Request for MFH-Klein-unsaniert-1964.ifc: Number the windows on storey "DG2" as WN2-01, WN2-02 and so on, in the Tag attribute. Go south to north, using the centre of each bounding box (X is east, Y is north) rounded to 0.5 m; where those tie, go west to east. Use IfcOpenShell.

First a look at what the model holds.

```python
import ifcopenshell
import ifcopenshell.util.element
import ifcopenshell.util.placement

model = ifcopenshell.open("MFH-Klein-unsaniert-1964.ifc")
print(model.schema)
storey = next(s for s in model.by_type("IfcBuildingStorey") if s.Name == "DG2")
windows = [e for e in ifcopenshell.util.element.get_decomposition(storey) if e.is_a("IfcWindow")]
for e in sorted(windows, key=lambda e: e.id()):
    origin = ifcopenshell.util.placement.get_local_placement(e.ObjectPlacement)[:3, 3]
    print(e.id(), e.Tag, e.Name, origin.round(2) + 0.0, sep=" | ")
```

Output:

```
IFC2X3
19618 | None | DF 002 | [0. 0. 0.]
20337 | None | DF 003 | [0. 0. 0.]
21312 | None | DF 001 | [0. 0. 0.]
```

```python
import ifcopenshell
import ifcopenshell.geom
import ifcopenshell.util.element
import ifcopenshell.util.shape

model = ifcopenshell.open("MFH-Klein-unsaniert-1964.ifc")
settings = ifcopenshell.geom.settings()
settings.set("use-world-coords", True)


def centre(element):
    shape = ifcopenshell.geom.create_shape(settings, element)
    return ifcopenshell.util.shape.get_bbox_centroid(shape.geometry)


storey = next(s for s in model.by_type("IfcBuildingStorey") if s.Name == "DG2")
windows = [e for e in ifcopenshell.util.element.get_decomposition(storey) if e.is_a("IfcWindow")]

# Insertion points can sit at a corner or the storey origin, so sort by the geometry (in metres).
centres = {e: centre(e) for e in windows}
windows.sort(key=lambda e: (round(centres[e][1] / 0.5), centres[e][0]))

for i, e in enumerate(windows, start=1):
    number = f"WN2-{i:02d}"
    e.Tag = number
    print(e.id(), number)

model.write("MFH-Klein-unsaniert-1964-out.ifc")
```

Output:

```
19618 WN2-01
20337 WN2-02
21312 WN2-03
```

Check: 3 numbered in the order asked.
